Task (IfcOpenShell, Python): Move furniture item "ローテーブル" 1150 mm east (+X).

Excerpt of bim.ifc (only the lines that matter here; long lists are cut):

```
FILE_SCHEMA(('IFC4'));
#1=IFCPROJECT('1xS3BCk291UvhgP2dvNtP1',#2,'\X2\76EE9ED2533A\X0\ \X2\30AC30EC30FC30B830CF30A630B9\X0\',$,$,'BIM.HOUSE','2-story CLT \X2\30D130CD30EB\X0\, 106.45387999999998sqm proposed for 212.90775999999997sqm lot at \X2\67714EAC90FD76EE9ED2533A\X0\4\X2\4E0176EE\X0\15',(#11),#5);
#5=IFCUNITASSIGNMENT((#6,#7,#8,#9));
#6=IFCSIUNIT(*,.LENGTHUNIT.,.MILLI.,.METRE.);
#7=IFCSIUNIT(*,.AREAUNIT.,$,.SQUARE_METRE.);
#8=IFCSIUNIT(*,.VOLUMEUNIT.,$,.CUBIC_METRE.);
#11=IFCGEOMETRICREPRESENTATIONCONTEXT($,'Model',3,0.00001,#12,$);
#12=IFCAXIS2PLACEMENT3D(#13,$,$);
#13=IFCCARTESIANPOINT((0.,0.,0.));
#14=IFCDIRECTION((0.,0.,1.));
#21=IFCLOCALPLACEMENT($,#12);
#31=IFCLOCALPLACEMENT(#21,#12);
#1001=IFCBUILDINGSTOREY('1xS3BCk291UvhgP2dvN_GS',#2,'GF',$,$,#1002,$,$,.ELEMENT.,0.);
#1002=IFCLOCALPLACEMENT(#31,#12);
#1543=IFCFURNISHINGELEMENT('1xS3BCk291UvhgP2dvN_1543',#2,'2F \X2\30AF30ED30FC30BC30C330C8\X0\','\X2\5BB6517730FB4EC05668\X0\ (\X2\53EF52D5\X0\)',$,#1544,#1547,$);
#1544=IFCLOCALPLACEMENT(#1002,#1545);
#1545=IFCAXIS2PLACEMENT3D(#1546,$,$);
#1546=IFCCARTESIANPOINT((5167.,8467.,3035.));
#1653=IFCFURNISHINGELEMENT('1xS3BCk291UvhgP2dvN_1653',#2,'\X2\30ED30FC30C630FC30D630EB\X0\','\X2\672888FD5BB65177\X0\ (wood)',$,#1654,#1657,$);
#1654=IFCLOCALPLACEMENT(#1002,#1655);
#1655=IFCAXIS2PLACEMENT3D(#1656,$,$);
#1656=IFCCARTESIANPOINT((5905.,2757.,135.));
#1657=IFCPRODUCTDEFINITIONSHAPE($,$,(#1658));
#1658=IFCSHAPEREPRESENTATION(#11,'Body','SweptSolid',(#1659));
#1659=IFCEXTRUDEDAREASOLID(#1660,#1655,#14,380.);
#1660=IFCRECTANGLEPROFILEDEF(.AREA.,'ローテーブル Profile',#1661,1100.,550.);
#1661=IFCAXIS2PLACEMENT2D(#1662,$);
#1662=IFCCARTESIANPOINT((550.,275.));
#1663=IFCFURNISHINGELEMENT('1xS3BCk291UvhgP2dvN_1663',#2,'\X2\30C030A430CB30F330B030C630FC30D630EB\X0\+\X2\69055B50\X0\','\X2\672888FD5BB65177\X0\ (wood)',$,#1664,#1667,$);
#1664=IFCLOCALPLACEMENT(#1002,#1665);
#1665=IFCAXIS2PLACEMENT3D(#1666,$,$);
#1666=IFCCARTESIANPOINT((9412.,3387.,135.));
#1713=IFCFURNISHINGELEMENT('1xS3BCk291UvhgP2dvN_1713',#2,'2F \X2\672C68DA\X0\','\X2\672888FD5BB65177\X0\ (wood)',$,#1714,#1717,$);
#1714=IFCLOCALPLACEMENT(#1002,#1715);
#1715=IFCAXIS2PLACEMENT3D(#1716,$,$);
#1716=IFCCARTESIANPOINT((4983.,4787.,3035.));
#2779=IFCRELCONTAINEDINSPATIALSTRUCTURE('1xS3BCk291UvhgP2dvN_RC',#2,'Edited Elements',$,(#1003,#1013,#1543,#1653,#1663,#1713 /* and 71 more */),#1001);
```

```python
import ifcopenshell
import ifcopenshell.api.geometry
import ifcopenshell.util.placement
import ifcopenshell.util.unit

model = ifcopenshell.open("bim.ifc")
unit_scale = ifcopenshell.util.unit.calculate_unit_scale(model)

item = model.by_guid("1xS3BCk291UvhgP2dvN_1653")
matrix = ifcopenshell.util.placement.get_local_placement(item.ObjectPlacement)
matrix[0, 3] += 1.15 / unit_scale
ifcopenshell.api.geometry.edit_object_placement(model, product=item, matrix=matrix, is_si=False)

print(ifcopenshell.util.placement.get_local_placement(item.ObjectPlacement).round(3) + 0.0)

model.write("bim_v2.ifc")
```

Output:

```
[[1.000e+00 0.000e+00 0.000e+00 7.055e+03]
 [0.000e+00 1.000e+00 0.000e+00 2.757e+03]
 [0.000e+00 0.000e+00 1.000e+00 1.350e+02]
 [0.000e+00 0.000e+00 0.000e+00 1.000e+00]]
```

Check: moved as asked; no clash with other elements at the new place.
